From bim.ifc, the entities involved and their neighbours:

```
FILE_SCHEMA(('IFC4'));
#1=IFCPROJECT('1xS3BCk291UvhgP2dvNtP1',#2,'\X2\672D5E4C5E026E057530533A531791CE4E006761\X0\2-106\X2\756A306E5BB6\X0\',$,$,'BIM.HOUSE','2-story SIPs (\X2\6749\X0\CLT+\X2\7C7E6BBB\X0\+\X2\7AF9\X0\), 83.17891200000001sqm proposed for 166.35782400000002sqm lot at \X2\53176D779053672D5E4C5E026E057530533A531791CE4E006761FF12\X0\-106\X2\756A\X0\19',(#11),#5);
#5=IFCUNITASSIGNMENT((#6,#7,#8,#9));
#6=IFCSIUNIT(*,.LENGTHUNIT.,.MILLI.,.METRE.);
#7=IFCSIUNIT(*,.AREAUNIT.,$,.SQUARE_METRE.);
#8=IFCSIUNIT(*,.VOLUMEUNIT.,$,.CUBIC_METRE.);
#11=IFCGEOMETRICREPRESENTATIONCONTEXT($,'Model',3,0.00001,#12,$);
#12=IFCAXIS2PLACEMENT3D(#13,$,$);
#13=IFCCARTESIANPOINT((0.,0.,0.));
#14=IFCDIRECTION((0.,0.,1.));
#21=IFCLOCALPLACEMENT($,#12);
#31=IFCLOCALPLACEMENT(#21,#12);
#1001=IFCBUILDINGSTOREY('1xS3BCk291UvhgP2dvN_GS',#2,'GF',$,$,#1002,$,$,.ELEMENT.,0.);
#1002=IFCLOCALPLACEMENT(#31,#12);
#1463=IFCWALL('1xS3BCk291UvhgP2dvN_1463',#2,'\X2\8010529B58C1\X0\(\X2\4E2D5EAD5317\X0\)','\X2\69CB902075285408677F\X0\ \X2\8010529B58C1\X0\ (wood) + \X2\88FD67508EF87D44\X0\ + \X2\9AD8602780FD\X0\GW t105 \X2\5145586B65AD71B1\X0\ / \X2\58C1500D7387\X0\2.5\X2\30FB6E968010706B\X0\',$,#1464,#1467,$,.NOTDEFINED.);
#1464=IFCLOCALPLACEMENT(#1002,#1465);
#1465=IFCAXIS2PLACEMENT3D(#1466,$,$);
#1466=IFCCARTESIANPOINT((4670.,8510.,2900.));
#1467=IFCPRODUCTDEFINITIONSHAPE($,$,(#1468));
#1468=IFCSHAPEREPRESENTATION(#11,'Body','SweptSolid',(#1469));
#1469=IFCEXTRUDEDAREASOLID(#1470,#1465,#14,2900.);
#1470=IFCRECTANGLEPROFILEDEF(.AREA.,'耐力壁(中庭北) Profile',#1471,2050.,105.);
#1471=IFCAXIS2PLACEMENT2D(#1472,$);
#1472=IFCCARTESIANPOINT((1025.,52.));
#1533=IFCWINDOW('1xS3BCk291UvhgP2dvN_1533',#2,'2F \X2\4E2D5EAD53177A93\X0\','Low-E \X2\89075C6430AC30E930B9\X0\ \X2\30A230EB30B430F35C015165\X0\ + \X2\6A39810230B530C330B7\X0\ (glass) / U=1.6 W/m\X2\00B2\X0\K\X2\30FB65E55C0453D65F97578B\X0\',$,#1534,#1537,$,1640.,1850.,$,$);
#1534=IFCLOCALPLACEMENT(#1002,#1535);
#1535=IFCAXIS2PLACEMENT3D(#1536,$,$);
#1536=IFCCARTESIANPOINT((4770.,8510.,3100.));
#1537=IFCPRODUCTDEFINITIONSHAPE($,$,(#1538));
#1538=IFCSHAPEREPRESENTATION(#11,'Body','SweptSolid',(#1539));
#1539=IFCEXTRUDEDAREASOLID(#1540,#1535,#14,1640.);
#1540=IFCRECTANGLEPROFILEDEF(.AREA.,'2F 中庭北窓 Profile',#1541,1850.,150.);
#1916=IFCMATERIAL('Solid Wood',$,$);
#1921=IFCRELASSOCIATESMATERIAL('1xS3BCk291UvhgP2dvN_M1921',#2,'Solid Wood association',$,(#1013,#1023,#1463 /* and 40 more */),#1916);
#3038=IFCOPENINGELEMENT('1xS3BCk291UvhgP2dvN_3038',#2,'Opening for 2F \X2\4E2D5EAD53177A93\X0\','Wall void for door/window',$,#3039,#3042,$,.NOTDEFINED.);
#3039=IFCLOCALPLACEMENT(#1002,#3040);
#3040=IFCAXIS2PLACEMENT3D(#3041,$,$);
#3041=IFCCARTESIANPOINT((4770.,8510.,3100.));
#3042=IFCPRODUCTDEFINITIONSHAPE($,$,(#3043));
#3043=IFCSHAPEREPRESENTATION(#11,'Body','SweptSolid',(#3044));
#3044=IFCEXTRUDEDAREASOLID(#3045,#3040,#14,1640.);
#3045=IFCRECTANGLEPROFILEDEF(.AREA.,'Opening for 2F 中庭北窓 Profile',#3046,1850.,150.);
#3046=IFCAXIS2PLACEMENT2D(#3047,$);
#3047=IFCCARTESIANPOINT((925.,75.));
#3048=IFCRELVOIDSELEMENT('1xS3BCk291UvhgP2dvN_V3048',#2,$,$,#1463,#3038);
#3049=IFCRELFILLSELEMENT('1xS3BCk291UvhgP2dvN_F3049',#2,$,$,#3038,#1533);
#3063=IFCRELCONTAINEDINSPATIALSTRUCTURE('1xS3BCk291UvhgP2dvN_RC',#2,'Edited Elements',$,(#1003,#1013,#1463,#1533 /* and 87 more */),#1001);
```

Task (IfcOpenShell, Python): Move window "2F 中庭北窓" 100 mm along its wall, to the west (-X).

```python
import ifcopenshell
import ifcopenshell.api.geometry
import ifcopenshell.util.placement
import ifcopenshell.util.unit

model = ifcopenshell.open("bim.ifc")
unit_scale = ifcopenshell.util.unit.calculate_unit_scale(model)

window = model.by_guid("1xS3BCk291UvhgP2dvN_1533")
opening = window.FillsVoids[0].RelatingOpeningElement
wall = opening.VoidsElements[0].RelatingBuildingElement

wall_matrix = ifcopenshell.util.placement.get_local_placement(wall.ObjectPlacement)
shift = wall_matrix[:3, 0] * -0.1 / unit_scale
before = ifcopenshell.util.placement.get_local_placement(window.ObjectPlacement)[:3, 3].copy()

# The window is not placed relative to its opening, so move both.
for product in (opening, window):
    matrix = ifcopenshell.util.placement.get_local_placement(product.ObjectPlacement)
    matrix[:3, 3] += shift
    ifcopenshell.api.geometry.edit_object_placement(model, product=product, matrix=matrix, is_si=False)

after = ifcopenshell.util.placement.get_local_placement(window.ObjectPlacement)[:3, 3]
print("window moved by", (after - before).round(3) + 0.0)

model.write("bim-out.ifc")
```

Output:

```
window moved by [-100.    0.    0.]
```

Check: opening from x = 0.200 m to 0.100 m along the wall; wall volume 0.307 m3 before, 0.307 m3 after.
